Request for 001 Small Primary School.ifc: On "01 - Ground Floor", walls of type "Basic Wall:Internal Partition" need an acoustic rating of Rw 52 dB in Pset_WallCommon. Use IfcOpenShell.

First a look at what the model holds.

```python
import ifcopenshell
import ifcopenshell.util.element

model = ifcopenshell.open("001 Small Primary School.ifc")
print(model.schema)
storey = next(s for s in model.by_type("IfcBuildingStorey") if s.Name == "01 - Ground Floor")
walls = [e for e in ifcopenshell.util.element.get_decomposition(storey) if e.is_a("IfcWall")]
seen = {}
for e in walls:
    element_type = ifcopenshell.util.element.get_type(e)
    key = (element_type.Name if element_type != e and element_type else None, ifcopenshell.util.element.get_pset(e, "Pset_WallCommon", "AcousticRating"))
    seen[key] = seen.get(key, 0) + 1
for (name, value), count in sorted(seen.items(), key=str):
    print(count, "x", name, "|", value)
```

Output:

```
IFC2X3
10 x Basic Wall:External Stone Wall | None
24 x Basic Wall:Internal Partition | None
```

```python
import ifcopenshell
import ifcopenshell.api.pset
import ifcopenshell.util.element

model = ifcopenshell.open("001 Small Primary School.ifc")

storey = next(s for s in model.by_type("IfcBuildingStorey") if s.Name == "01 - Ground Floor")
walls = [e for e in ifcopenshell.util.element.get_decomposition(storey) if e.is_a("IfcWall")]

count = 0
for e in walls:
    element_type = ifcopenshell.util.element.get_type(e)
    if element_type in (None, e) or element_type.Name != "Basic Wall:Internal Partition":
        continue
    # add_pset returns the element's existing set when there is one.
    pset = ifcopenshell.api.pset.add_pset(model, product=e, name="Pset_WallCommon")
    ifcopenshell.api.pset.edit_pset(model, pset=pset, properties={"AcousticRating": "Rw 52 dB"})
    count += 1

print(count, "walls updated")

model.write("001 Small Primary School_v2.ifc")
```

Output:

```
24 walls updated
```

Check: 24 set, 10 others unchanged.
